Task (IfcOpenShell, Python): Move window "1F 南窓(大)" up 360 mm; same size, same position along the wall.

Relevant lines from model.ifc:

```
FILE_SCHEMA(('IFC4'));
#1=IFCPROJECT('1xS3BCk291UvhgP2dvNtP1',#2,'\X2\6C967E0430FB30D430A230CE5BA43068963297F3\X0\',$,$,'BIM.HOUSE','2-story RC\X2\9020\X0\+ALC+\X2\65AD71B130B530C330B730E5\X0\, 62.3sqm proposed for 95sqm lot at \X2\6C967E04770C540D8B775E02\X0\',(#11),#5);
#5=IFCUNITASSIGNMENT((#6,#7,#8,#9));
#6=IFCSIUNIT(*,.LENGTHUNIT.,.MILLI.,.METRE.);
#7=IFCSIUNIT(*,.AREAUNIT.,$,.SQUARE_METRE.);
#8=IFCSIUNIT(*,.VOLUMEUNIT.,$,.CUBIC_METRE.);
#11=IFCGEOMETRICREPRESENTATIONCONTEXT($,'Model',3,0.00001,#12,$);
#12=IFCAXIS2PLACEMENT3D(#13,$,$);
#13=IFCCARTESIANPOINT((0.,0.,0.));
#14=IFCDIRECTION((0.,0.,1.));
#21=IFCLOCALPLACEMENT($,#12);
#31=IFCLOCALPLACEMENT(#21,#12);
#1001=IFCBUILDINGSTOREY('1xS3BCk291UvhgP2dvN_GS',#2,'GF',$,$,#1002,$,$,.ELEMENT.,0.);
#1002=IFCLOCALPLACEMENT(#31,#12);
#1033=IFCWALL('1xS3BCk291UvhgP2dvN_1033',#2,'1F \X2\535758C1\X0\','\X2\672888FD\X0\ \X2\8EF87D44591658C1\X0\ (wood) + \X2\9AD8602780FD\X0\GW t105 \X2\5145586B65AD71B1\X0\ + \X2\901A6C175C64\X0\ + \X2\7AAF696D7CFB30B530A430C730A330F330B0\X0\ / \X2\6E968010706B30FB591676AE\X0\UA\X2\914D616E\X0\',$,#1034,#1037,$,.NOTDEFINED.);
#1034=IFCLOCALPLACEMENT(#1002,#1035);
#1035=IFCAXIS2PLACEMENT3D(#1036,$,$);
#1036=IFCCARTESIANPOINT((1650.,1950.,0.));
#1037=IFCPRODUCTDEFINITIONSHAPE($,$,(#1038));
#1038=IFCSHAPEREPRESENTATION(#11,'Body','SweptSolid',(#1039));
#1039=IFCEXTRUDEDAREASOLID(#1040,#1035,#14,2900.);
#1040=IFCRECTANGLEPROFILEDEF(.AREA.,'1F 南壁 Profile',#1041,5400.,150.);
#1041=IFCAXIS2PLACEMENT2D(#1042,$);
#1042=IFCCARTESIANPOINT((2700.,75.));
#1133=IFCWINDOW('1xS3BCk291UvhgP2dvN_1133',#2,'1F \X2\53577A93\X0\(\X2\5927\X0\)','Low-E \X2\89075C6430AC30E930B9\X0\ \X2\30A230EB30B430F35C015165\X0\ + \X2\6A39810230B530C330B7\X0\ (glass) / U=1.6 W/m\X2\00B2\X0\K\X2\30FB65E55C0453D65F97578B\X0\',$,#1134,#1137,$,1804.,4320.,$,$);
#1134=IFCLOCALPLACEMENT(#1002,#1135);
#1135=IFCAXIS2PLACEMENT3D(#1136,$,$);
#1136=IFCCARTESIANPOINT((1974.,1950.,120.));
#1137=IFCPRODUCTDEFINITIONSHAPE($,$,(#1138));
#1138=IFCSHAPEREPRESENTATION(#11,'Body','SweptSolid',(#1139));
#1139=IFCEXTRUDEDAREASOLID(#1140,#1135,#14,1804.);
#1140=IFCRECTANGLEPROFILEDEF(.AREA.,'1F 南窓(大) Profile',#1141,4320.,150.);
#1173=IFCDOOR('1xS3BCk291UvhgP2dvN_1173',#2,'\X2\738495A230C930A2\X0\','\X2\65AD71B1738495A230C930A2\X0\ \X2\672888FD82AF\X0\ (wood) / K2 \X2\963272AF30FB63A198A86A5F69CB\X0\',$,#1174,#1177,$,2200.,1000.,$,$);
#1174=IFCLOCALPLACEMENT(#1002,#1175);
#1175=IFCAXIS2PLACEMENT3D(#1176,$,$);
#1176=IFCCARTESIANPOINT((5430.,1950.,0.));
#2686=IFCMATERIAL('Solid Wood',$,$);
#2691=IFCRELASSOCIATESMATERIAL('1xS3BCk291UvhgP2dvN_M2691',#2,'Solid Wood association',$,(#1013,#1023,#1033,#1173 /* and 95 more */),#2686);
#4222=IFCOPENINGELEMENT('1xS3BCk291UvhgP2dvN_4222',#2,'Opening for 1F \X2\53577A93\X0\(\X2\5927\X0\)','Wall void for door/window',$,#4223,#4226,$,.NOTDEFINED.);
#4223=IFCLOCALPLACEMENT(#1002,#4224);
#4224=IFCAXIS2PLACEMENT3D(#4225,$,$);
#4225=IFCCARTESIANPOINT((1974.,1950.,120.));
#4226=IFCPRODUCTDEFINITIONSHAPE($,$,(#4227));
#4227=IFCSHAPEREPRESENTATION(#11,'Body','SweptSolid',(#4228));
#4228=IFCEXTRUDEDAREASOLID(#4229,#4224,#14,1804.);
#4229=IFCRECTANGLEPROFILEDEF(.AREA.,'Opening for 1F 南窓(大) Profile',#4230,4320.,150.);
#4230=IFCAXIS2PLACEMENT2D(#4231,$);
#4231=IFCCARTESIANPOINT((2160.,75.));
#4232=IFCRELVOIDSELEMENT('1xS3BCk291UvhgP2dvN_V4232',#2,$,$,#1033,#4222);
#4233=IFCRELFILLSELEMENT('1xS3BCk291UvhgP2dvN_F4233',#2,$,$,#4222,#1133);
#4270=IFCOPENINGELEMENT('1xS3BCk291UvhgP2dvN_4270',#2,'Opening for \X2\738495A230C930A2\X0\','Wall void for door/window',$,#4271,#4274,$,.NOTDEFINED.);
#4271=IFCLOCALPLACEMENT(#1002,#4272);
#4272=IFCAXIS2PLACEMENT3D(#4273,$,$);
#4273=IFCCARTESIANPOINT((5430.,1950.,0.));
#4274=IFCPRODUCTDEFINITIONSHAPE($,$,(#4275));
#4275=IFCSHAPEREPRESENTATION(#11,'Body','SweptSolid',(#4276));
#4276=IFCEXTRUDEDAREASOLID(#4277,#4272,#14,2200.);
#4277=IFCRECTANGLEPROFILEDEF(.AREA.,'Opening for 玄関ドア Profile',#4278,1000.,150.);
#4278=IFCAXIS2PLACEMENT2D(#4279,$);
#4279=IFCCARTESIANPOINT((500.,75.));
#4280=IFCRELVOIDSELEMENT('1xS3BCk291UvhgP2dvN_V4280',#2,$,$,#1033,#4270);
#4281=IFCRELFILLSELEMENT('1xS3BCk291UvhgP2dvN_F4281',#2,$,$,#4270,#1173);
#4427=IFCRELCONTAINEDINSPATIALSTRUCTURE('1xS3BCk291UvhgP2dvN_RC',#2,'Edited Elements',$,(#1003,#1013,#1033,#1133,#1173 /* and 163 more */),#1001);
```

```python
import numpy as np
import ifcopenshell
import ifcopenshell.api.geometry
import ifcopenshell.util.placement
import ifcopenshell.util.unit

model = ifcopenshell.open("model.ifc")
unit_scale = ifcopenshell.util.unit.calculate_unit_scale(model)

window = model.by_id(1133)
opening = window.FillsVoids[0].RelatingOpeningElement
dz = 0.36 / unit_scale

shift = np.array([0.0, 0.0, dz])
# The window is not placed relative to its opening, so move both.
for product in (opening, window):
    matrix = ifcopenshell.util.placement.get_local_placement(product.ObjectPlacement)
    matrix[:3, 3] += shift
    ifcopenshell.api.geometry.edit_object_placement(model, product=product, matrix=matrix, is_si=False)

print(f"moved by {dz * unit_scale:+.3f} m")

model.write("model_v2.ifc")
```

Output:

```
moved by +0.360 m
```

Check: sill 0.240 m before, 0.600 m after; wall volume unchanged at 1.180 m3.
